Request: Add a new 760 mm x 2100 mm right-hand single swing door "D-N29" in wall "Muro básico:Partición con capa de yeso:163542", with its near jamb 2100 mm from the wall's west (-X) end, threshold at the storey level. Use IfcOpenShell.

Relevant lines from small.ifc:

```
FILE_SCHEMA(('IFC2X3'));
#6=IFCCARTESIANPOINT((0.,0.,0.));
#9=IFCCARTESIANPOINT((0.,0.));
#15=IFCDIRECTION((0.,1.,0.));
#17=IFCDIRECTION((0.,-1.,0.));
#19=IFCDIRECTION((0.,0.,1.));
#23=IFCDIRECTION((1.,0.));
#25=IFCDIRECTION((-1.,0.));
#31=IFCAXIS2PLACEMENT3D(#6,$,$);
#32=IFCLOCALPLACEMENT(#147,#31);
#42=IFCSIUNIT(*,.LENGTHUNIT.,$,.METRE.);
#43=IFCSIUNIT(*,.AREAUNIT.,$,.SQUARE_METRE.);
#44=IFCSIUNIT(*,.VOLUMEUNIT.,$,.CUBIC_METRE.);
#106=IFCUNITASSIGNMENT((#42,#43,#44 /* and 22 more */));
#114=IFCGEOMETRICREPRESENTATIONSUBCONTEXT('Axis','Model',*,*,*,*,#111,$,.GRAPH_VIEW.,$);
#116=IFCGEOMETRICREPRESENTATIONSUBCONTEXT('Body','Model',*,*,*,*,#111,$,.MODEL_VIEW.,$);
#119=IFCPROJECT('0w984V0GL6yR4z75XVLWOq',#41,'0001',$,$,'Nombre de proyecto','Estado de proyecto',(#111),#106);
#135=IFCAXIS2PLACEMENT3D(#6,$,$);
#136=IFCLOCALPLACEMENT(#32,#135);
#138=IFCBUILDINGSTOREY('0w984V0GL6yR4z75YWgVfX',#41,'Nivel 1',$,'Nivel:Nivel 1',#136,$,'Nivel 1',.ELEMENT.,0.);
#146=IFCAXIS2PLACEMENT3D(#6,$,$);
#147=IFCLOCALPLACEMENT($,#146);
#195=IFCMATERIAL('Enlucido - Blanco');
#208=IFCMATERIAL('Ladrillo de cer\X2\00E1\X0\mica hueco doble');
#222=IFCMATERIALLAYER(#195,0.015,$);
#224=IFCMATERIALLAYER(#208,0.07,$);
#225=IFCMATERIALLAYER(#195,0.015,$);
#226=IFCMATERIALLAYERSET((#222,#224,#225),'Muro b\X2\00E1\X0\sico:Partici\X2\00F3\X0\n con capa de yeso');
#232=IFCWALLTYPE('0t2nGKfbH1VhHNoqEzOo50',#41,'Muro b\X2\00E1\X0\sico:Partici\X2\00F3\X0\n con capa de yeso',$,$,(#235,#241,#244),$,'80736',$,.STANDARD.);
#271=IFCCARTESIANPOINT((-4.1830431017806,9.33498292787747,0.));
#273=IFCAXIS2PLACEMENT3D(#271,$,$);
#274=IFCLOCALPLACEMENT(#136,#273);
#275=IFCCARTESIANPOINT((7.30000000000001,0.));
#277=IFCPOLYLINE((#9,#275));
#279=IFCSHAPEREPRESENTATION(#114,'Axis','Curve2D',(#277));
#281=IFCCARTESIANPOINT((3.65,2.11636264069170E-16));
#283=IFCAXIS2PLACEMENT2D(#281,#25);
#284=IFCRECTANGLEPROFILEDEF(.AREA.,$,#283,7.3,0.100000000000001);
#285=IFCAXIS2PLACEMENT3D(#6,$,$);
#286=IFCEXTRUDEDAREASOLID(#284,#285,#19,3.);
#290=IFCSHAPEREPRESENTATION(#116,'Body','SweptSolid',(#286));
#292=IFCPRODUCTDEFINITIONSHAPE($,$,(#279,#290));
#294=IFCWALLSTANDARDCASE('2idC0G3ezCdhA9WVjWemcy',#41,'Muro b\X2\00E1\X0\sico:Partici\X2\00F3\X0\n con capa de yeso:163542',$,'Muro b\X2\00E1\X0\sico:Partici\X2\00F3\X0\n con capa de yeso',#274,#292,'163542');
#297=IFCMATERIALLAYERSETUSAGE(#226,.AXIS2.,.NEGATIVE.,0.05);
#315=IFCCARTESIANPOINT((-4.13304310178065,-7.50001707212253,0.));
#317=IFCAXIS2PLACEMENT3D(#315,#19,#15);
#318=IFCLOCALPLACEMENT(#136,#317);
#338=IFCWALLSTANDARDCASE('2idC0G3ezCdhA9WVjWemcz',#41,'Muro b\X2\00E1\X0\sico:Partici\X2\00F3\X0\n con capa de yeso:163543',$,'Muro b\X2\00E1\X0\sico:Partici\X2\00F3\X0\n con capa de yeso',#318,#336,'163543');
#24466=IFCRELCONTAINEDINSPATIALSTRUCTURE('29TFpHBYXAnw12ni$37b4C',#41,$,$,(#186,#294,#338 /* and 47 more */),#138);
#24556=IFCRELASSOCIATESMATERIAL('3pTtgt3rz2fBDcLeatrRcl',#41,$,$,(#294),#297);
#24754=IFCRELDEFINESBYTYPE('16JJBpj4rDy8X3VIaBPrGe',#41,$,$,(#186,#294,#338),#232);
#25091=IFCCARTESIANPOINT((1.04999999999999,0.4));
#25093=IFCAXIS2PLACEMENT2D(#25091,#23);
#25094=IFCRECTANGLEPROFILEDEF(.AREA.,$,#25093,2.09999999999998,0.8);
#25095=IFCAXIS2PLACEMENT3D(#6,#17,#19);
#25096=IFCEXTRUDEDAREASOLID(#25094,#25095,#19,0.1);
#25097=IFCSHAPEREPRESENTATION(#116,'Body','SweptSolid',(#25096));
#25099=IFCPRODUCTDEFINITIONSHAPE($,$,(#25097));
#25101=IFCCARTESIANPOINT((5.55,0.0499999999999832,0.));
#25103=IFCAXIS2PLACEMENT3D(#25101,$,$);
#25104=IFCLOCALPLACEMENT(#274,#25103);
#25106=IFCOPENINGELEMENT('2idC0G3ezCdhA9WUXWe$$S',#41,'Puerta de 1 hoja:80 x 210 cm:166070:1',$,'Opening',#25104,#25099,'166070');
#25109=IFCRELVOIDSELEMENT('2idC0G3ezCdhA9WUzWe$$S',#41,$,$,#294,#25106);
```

```python
import numpy as np
import ifcopenshell
import ifcopenshell.api.feature
import ifcopenshell.api.geometry
import ifcopenshell.api.root
import ifcopenshell.api.spatial
import ifcopenshell.api.type
import ifcopenshell.geom
import ifcopenshell.util.element
import ifcopenshell.util.placement
import ifcopenshell.util.representation
import ifcopenshell.util.shape
import ifcopenshell.util.unit

model = ifcopenshell.open("small.ifc")
unit_scale = ifcopenshell.util.unit.calculate_unit_scale(model)
settings = ifcopenshell.geom.settings()


def volume(element):
    """Net volume in cubic metres, openings subtracted."""
    shape = ifcopenshell.geom.create_shape(settings, element)
    return ifcopenshell.util.shape.get_volume(shape.geometry)


wall = model.by_id(294)
storey = ifcopenshell.util.element.get_container(wall, ifc_class="IfcBuildingStorey")
context = ifcopenshell.util.representation.get_context(model, "Model", "Body", "MODEL_VIEW")
before = volume(wall)

width, height, from_end, sill = 0.76, 2.1, 2.1, 0.0  # metres

# The wall runs along its own X axis, and the end named is its -X end.
wall_shape = ifcopenshell.geom.create_shape(settings, wall)
x, y, z = ifcopenshell.util.shape.get_vertices(wall_shape.geometry).T
start = x.min() + from_end
face, thickness = float(y.min()), float(y.max() - y.min())
wall_matrix = ifcopenshell.util.placement.get_local_placement(wall.ObjectPlacement)
level = ifcopenshell.util.placement.get_local_placement(storey.ObjectPlacement)[2, 3]


def in_wall(x, y):
    """Placement at x, y metres in the wall's axes, at sill height."""
    matrix = wall_matrix.copy()
    matrix[:, 3] = wall_matrix @ np.array([x / unit_scale, y / unit_scale, 0.0, 1.0])
    matrix[2, 3] = level + sill / unit_scale
    return matrix


# Opening: a box that overshoots both wall faces by 50 mm.
opening = ifcopenshell.api.root.create_entity(model, ifc_class="IfcOpeningElement")
box = ifcopenshell.api.geometry.add_wall_representation(
    model, context=context, length=width, height=height, thickness=thickness + 0.1
)
ifcopenshell.api.geometry.assign_representation(model, product=opening, representation=box)
ifcopenshell.api.geometry.edit_object_placement(model, product=opening, matrix=in_wall(start, face - 0.05), is_si=False)
ifcopenshell.api.feature.add_feature(model, feature=opening, element=wall)

door = ifcopenshell.api.root.create_entity(model, ifc_class="IfcDoor", name="D-N29")
door.OverallWidth, door.OverallHeight = width / unit_scale, height / unit_scale
body = ifcopenshell.api.geometry.add_door_representation(
    model,
    context=context,
    overall_width=door.OverallWidth,
    overall_height=door.OverallHeight,
    operation_type="SINGLE_SWING_RIGHT",
    lining_properties={"LiningDepth": thickness / unit_scale, "ThresholdDepth": thickness / unit_scale},
)
ifcopenshell.api.geometry.assign_representation(model, product=door, representation=body)
ifcopenshell.api.spatial.assign_container(model, products=[door], relating_structure=storey)
fills = ifcopenshell.api.feature.add_filling(model, opening=opening, element=door)
fills.OwnerHistory = door.OwnerHistory  # required in IFC2X3

# IFC2X3 keeps the operation on the door style.
style = ifcopenshell.api.root.create_entity(model, ifc_class="IfcDoorStyle", name="D-N29")
style.OperationType, style.ConstructionType = "SINGLE_SWING_RIGHT", "NOTDEFINED"
style.ParameterTakesPrecedence = style.Sizeable = False
ifcopenshell.api.type.assign_type(model, related_objects=[door], relating_type=style)

# The lining spans the wall, so the door starts at the wall face.
ifcopenshell.api.geometry.edit_object_placement(model, product=door, matrix=in_wall(start, face), is_si=False)

after = volume(wall)

print(f"wall volume {before:.3f} -> {after:.3f} m3")

model.write("small_v2.ifc")
```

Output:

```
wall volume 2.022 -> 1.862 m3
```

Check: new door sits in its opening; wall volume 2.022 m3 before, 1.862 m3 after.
